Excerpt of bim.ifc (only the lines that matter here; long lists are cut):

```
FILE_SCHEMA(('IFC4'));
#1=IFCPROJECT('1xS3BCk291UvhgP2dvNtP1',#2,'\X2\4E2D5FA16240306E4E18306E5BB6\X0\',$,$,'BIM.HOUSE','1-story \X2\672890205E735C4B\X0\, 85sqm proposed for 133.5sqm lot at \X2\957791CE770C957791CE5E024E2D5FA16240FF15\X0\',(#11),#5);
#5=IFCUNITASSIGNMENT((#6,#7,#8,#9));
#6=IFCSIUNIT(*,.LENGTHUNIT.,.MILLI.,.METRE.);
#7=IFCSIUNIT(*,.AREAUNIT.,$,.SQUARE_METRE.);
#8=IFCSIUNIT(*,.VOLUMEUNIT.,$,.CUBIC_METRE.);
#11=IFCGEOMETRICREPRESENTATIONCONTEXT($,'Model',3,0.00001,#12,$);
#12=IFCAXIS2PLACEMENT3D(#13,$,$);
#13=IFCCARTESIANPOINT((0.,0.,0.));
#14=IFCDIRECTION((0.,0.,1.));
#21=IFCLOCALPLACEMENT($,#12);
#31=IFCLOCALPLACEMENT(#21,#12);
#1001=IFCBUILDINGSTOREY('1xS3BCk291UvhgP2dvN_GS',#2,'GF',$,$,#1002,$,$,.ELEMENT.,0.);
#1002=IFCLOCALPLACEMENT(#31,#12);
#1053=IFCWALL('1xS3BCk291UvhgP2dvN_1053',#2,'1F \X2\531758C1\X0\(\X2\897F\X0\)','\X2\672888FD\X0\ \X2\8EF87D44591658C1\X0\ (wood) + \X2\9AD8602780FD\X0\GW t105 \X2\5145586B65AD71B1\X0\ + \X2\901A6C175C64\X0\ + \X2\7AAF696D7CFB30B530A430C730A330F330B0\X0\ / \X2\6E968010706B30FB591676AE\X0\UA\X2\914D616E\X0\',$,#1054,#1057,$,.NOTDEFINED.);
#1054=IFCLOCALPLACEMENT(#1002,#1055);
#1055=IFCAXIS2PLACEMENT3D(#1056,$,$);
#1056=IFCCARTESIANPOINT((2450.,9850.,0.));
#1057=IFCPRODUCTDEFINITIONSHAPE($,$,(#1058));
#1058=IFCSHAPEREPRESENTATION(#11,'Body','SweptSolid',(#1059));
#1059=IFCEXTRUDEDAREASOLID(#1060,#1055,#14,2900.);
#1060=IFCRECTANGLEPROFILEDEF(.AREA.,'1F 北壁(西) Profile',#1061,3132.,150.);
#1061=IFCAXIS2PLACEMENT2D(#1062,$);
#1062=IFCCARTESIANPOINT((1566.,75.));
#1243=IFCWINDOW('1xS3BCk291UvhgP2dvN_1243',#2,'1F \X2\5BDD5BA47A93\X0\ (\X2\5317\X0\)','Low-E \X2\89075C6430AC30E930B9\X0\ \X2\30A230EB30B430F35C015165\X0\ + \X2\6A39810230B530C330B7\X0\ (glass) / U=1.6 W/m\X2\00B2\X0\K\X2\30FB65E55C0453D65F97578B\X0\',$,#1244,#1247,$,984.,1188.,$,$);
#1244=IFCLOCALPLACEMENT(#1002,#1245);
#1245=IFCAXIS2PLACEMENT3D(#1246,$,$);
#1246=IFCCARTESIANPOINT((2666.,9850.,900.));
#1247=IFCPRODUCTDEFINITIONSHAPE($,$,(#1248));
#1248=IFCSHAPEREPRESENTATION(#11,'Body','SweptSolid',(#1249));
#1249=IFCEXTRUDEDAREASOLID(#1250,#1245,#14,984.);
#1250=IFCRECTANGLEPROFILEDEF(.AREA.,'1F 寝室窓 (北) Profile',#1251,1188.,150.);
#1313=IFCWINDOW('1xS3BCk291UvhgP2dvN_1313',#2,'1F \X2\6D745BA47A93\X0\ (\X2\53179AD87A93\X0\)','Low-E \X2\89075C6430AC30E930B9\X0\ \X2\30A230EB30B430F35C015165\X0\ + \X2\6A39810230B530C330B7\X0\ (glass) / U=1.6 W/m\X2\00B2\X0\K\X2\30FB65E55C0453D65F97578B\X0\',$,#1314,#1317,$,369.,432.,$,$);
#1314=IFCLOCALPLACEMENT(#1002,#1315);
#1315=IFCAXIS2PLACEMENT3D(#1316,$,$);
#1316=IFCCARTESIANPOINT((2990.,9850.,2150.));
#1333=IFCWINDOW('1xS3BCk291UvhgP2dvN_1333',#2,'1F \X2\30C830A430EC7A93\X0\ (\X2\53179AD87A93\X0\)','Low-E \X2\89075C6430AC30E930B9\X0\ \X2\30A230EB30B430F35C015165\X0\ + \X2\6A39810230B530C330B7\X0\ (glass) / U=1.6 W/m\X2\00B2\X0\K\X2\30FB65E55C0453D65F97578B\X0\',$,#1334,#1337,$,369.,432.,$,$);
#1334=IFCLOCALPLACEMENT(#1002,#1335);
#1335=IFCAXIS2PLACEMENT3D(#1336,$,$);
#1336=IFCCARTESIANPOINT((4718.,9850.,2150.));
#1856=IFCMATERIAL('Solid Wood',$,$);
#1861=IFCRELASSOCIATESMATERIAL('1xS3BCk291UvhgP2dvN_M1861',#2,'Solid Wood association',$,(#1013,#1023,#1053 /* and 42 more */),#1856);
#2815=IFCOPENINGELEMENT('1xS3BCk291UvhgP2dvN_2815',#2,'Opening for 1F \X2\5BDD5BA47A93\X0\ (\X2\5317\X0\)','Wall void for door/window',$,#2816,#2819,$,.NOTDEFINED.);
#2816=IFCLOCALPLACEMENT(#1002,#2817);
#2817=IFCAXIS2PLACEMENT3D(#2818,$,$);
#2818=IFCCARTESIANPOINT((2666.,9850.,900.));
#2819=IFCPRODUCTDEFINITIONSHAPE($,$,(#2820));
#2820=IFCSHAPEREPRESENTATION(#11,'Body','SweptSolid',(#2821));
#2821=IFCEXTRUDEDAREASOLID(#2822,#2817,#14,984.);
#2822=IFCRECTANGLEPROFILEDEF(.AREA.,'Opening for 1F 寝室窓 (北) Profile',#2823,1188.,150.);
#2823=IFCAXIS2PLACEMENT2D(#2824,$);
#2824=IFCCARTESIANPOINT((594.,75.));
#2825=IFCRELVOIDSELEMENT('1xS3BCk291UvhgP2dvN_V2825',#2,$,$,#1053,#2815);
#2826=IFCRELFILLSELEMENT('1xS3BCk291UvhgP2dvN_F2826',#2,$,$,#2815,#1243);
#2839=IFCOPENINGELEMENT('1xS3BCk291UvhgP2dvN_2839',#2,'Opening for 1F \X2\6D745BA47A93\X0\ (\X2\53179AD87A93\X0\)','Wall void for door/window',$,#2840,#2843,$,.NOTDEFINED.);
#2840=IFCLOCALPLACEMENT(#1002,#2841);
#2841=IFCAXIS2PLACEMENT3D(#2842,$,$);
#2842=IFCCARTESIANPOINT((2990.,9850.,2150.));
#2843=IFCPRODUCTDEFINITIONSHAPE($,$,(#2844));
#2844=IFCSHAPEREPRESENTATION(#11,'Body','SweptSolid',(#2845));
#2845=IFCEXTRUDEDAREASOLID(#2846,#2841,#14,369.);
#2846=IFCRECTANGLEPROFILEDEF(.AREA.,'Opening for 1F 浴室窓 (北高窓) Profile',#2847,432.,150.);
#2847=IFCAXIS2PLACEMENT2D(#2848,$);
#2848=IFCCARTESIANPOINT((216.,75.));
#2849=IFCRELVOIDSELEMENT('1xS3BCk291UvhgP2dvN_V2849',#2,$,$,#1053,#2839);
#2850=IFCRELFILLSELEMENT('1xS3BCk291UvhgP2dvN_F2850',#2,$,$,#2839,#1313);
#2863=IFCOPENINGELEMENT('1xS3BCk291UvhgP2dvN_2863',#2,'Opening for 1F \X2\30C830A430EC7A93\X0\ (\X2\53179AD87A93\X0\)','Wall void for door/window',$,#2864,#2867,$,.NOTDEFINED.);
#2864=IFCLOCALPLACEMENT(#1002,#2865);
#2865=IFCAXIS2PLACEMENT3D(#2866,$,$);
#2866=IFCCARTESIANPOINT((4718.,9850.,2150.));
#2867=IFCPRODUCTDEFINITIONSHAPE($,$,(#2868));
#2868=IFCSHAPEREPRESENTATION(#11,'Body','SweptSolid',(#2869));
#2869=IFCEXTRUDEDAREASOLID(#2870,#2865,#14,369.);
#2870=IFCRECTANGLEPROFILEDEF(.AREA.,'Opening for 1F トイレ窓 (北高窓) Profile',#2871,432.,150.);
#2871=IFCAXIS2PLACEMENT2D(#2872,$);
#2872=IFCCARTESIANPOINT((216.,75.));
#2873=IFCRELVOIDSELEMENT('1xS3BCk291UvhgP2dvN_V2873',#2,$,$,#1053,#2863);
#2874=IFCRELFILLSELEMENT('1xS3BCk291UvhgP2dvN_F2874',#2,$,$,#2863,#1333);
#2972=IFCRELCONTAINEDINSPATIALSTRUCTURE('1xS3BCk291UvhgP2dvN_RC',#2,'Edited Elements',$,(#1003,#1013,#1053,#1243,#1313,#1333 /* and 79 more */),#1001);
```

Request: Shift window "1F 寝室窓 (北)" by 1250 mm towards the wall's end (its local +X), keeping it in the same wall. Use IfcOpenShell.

```python
import ifcopenshell
import ifcopenshell.api.geometry
import ifcopenshell.util.placement

model = ifcopenshell.open("bim.ifc")

window = model.by_id(1243)
opening = window.FillsVoids[0].RelatingOpeningElement
wall = opening.VoidsElements[0].RelatingBuildingElement

wall_matrix = ifcopenshell.util.placement.get_local_placement(wall.ObjectPlacement)
shift = wall_matrix[:3, 0] * 1250.0
before = ifcopenshell.util.placement.get_local_placement(window.ObjectPlacement)[:3, 3].copy()

# The window is not placed relative to its opening, so move both.
for product in (opening, window):
    matrix = ifcopenshell.util.placement.get_local_placement(product.ObjectPlacement)
    matrix[:3, 3] += shift
    ifcopenshell.api.geometry.edit_object_placement(model, product=product, matrix=matrix, is_si=False)

after = ifcopenshell.util.placement.get_local_placement(window.ObjectPlacement)[:3, 3]
print("window moved by", (after - before).round(3) + 0.0)

model.write("bim_updated.ifc")
```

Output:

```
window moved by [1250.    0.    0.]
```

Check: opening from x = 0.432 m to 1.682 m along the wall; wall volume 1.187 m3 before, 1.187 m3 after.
